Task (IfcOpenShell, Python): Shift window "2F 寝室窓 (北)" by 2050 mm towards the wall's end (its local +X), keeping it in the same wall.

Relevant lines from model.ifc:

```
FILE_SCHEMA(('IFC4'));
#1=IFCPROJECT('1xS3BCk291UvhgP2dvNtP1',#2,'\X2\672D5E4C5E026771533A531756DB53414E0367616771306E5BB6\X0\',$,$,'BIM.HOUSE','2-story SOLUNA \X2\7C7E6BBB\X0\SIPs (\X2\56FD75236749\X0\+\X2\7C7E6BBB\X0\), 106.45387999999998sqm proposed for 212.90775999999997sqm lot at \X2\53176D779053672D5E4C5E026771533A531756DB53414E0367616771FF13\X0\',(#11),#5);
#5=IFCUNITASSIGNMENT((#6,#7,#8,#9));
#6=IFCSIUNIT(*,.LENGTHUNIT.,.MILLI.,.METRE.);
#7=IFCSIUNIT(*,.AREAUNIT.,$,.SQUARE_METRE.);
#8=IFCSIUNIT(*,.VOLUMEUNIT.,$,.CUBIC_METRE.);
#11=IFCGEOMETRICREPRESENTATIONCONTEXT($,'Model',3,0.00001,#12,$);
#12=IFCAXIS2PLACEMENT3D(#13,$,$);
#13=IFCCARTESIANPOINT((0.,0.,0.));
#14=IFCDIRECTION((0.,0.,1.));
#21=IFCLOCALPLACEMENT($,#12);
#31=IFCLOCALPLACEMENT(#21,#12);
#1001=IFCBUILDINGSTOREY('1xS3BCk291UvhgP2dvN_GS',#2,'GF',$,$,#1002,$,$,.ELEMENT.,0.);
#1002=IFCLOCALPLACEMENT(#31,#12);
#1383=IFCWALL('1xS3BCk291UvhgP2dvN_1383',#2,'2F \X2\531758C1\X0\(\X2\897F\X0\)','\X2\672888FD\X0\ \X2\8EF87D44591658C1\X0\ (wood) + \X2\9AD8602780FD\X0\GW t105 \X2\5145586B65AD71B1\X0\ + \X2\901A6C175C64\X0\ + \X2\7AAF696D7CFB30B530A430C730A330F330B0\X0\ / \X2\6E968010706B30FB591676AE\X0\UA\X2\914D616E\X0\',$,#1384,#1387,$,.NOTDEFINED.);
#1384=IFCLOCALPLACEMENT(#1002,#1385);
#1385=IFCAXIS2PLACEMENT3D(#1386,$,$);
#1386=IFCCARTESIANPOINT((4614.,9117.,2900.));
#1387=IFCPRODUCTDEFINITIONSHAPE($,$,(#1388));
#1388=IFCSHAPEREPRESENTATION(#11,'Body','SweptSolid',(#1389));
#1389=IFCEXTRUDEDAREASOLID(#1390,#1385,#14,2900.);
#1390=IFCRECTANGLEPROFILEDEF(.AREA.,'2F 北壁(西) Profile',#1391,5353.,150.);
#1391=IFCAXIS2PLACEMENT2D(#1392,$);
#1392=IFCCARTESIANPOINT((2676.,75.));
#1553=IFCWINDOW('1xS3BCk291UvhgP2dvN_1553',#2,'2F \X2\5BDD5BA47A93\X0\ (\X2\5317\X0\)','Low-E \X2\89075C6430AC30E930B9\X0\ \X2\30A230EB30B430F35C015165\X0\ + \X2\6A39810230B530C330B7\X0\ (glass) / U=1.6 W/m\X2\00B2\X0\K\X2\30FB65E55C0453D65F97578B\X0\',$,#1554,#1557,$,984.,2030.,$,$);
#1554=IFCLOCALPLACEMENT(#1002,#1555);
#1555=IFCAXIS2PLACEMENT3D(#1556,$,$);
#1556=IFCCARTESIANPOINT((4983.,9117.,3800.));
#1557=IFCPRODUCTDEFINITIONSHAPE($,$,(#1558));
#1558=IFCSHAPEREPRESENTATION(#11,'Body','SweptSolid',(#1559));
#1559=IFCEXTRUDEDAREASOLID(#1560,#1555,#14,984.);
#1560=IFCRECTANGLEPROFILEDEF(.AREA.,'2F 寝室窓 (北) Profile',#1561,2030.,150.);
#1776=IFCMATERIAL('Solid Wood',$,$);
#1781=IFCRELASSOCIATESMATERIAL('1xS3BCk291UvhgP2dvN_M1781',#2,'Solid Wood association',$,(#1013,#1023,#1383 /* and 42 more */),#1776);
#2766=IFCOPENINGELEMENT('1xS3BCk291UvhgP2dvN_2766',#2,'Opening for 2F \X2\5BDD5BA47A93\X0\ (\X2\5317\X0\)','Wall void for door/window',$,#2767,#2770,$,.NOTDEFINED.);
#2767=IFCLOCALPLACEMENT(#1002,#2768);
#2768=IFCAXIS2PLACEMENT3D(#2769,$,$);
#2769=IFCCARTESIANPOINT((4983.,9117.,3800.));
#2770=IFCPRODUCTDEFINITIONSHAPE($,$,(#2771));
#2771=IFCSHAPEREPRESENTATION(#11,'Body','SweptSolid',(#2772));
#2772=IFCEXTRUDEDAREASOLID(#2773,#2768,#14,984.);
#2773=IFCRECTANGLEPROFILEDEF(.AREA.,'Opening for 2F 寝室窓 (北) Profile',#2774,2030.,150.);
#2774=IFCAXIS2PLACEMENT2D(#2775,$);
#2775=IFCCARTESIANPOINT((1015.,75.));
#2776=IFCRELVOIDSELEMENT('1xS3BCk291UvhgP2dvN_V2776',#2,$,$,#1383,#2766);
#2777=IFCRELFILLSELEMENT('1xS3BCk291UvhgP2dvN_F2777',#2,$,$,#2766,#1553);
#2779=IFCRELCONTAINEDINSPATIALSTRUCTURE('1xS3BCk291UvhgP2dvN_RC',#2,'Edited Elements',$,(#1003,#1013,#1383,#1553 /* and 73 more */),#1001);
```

```python
import ifcopenshell
import ifcopenshell.api.geometry
import ifcopenshell.util.placement
import ifcopenshell.util.unit

model = ifcopenshell.open("model.ifc")
unit_scale = ifcopenshell.util.unit.calculate_unit_scale(model)

window = model.by_id(1553)
opening = window.FillsVoids[0].RelatingOpeningElement
wall = opening.VoidsElements[0].RelatingBuildingElement

wall_matrix = ifcopenshell.util.placement.get_local_placement(wall.ObjectPlacement)
shift = wall_matrix[:3, 0] * 2.05 / unit_scale
before = ifcopenshell.util.placement.get_local_placement(window.ObjectPlacement)[:3, 3].copy()

# The window is not placed relative to its opening, so move both.
for product in (opening, window):
    matrix = ifcopenshell.util.placement.get_local_placement(product.ObjectPlacement)
    matrix[:3, 3] += shift
    ifcopenshell.api.geometry.edit_object_placement(model, product=product, matrix=matrix, is_si=False)

after = ifcopenshell.util.placement.get_local_placement(window.ObjectPlacement)[:3, 3]
print("window moved by", (after - before).round(3) + 0.0)

model.write("model_rev.ifc")
```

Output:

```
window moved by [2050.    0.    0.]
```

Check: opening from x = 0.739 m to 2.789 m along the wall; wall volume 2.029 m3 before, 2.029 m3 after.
